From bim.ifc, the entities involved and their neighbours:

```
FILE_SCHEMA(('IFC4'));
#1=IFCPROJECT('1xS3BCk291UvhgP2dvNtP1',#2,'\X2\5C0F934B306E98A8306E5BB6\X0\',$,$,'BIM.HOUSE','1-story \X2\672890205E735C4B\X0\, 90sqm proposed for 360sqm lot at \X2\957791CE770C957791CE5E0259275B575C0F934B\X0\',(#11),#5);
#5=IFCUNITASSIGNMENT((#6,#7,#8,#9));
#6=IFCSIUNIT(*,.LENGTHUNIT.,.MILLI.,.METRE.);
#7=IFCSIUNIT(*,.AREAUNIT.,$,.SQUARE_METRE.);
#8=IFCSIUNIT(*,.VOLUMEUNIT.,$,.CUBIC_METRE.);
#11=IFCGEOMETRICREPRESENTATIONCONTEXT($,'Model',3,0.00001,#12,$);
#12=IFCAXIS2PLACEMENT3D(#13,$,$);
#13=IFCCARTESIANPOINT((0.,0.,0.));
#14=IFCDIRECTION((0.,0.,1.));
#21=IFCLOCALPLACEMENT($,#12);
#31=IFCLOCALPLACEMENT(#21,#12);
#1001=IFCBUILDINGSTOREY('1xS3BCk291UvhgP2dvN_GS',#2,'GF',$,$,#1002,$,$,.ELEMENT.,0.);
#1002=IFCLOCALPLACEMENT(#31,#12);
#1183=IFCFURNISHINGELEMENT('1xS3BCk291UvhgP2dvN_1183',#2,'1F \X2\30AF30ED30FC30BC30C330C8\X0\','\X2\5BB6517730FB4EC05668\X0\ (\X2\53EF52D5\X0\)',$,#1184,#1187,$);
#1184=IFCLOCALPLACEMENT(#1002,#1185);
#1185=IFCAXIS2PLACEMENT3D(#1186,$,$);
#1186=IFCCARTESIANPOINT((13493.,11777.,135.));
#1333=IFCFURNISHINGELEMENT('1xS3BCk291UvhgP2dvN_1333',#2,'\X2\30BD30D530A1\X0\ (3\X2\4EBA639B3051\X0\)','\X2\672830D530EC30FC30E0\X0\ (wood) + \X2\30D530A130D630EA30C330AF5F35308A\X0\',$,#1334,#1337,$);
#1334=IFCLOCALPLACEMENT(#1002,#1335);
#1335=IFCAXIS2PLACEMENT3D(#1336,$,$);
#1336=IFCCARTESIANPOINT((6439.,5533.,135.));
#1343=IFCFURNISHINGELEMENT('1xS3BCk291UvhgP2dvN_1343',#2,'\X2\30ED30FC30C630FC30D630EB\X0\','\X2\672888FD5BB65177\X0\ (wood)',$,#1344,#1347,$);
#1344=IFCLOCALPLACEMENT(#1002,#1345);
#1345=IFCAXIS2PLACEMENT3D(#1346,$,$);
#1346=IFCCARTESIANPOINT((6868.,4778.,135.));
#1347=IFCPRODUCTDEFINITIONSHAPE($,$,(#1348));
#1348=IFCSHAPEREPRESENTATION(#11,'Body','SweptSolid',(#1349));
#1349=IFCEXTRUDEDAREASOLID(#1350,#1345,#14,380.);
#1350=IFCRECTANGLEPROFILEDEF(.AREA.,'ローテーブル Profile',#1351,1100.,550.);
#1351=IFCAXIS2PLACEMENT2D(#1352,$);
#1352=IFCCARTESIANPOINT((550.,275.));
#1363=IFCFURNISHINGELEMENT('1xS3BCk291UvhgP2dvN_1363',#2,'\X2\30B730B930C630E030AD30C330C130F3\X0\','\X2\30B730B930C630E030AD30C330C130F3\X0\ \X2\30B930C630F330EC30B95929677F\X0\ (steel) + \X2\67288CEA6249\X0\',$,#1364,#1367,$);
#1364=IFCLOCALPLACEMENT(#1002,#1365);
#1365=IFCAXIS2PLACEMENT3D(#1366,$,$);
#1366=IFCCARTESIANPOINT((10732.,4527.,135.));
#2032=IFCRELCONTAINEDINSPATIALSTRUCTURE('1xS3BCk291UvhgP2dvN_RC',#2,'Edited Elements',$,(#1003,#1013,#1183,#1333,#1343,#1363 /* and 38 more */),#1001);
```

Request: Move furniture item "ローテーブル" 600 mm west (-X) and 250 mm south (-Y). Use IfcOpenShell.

```python
import ifcopenshell
import ifcopenshell.api.geometry
import ifcopenshell.util.placement
import ifcopenshell.util.unit

model = ifcopenshell.open("bim.ifc")
unit_scale = ifcopenshell.util.unit.calculate_unit_scale(model)

item = model.by_guid("1xS3BCk291UvhgP2dvN_1343")
matrix = ifcopenshell.util.placement.get_local_placement(item.ObjectPlacement)
matrix[0, 3] -= 0.6 / unit_scale
matrix[1, 3] -= 0.25 / unit_scale
ifcopenshell.api.geometry.edit_object_placement(model, product=item, matrix=matrix, is_si=False)

print(ifcopenshell.util.placement.get_local_placement(item.ObjectPlacement).round(3) + 0.0)

model.write("bim_edited.ifc")
```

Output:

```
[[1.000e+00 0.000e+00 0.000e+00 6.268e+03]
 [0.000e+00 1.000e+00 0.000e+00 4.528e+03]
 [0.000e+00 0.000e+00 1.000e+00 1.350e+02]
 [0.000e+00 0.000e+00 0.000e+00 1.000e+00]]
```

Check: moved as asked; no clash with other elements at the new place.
